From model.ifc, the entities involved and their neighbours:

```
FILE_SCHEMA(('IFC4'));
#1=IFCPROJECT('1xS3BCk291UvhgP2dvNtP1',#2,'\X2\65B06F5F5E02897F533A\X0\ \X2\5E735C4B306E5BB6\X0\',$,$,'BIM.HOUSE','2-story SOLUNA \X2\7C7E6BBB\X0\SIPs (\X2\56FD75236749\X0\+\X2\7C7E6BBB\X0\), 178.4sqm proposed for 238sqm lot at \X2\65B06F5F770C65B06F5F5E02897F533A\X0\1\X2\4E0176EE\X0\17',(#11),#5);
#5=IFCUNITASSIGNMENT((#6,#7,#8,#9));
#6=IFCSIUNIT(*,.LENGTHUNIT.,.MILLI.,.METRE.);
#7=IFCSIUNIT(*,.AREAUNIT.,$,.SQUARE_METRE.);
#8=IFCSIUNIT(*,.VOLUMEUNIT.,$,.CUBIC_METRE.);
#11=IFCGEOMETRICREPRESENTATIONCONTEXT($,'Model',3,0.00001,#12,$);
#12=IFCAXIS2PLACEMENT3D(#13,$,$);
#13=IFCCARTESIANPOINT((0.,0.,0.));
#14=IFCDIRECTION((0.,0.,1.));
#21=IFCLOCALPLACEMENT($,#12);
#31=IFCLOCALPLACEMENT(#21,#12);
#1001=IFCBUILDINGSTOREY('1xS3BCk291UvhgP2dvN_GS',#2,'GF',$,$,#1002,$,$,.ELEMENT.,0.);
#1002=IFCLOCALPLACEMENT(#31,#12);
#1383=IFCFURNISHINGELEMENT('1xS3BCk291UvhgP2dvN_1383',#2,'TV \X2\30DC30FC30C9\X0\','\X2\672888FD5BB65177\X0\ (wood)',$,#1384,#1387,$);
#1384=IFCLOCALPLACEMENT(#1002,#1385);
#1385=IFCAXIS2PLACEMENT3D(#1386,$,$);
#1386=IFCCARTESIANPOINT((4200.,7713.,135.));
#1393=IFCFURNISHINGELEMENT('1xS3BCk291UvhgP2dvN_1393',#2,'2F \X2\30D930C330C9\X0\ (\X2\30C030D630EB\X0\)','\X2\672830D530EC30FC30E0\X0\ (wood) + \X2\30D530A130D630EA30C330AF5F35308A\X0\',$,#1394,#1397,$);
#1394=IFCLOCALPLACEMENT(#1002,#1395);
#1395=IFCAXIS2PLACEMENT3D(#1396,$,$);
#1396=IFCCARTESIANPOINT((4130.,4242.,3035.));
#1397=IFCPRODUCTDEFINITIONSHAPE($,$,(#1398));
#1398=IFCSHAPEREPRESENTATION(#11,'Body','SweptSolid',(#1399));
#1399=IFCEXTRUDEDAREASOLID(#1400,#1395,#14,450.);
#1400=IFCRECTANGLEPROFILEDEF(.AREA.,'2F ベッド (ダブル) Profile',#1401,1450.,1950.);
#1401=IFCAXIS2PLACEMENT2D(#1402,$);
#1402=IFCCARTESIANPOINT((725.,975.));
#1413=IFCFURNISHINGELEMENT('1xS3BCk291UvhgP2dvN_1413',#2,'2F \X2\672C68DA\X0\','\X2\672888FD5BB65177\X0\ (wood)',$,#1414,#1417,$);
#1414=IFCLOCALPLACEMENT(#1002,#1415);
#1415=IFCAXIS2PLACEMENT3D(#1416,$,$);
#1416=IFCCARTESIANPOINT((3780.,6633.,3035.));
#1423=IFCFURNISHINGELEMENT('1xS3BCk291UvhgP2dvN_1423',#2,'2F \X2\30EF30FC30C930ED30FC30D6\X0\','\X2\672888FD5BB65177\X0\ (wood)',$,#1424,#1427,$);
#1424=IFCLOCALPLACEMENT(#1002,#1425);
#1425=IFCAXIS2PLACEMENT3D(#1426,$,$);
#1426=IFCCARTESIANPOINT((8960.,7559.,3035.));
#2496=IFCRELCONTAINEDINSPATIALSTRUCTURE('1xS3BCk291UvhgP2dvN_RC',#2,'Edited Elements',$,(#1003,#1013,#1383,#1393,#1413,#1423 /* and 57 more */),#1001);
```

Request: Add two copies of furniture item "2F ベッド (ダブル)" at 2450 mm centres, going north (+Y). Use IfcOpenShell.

```python
import numpy as np
import ifcopenshell
import ifcopenshell.api.geometry
import ifcopenshell.api.root
import ifcopenshell.util.element
import ifcopenshell.util.placement
import ifcopenshell.util.unit

model = ifcopenshell.open("model.ifc")
unit_scale = ifcopenshell.util.unit.calculate_unit_scale(model)


def reuse_history(source, copy):
    """copy_class also copies each property set's owner history, people and application; keep the originals."""
    for rel in copy.IsDefinedBy:
        if rel.is_a("IfcRelDefinesByProperties") and (history := rel.RelatingPropertyDefinition.OwnerHistory):
            rel.RelatingPropertyDefinition.OwnerHistory = source.OwnerHistory
            ifcopenshell.util.element.remove_deep2(model, history)


source = model.by_guid("1xS3BCk291UvhgP2dvN_1393")
base = ifcopenshell.util.placement.get_local_placement(source.ObjectPlacement)
step = np.array([0.0, 1.0, 0.0]) * 2.45 / unit_scale

for i in range(1, 3):
    copy = ifcopenshell.api.root.copy_class(model, product=source)
    copy.Representation = ifcopenshell.util.element.copy_deep(
        model, source.Representation, exclude=["IfcGeometricRepresentationContext", "IfcRepresentationMap"]
    )
    reuse_history(source, copy)
    matrix = base.copy()
    matrix[:3, 3] += i * step
    print("added at", matrix[:3, 3].round(3) + 0.0)
    ifcopenshell.api.geometry.edit_object_placement(model, product=copy, matrix=matrix, is_si=False)

model.write("model_edited.ifc")
```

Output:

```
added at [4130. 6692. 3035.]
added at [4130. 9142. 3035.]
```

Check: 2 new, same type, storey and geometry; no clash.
